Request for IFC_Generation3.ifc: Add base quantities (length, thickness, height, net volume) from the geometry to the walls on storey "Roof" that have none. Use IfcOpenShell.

First a look at what the model holds.

```python
import ifcopenshell
import ifcopenshell.util.element
import ifcopenshell.util.unit

model = ifcopenshell.open("IFC_Generation3.ifc")
print(model.schema)
for unit_type in ("LENGTHUNIT", "AREAUNIT", "VOLUMEUNIT"):
    print(unit_type, ifcopenshell.util.unit.calculate_unit_scale(model, unit_type))
storey = next(s for s in model.by_type("IfcBuildingStorey") if s.Name == "Roof")
walls = [e for e in ifcopenshell.util.element.get_decomposition(storey) if e.is_a("IfcWall")]
for e in sorted(walls, key=lambda e: e.id()):
    print(e.id(), e.is_a(), e.Name, list(ifcopenshell.util.element.get_psets(e, qtos_only=True)), sep=" | ")
```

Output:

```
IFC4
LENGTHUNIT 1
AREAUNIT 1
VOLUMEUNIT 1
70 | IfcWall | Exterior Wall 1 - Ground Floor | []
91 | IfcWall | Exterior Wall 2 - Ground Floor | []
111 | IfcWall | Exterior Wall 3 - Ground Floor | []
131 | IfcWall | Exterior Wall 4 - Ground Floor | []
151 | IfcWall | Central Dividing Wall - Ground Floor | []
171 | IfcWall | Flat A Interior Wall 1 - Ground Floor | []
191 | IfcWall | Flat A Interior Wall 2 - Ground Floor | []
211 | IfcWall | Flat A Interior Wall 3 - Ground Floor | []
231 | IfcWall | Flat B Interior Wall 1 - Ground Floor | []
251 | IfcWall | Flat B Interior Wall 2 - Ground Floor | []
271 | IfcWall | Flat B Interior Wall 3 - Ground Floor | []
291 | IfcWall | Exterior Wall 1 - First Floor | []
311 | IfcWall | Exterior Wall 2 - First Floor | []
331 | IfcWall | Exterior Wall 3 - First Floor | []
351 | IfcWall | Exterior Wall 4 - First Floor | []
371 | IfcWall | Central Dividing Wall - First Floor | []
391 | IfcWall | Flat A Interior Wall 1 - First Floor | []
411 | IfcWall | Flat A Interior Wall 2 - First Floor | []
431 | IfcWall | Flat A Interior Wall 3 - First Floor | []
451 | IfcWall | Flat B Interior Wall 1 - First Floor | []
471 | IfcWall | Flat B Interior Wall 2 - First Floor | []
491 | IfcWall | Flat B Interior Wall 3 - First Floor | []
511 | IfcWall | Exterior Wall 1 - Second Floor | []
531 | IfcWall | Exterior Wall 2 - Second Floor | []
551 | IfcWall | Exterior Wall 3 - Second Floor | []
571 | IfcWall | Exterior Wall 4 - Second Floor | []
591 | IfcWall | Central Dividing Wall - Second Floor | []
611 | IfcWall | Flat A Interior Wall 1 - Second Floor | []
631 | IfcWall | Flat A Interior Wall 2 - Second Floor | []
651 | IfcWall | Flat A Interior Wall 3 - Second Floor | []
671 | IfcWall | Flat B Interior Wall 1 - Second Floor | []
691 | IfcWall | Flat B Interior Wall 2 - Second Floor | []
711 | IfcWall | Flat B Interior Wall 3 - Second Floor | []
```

```python
import ifcopenshell
import ifcopenshell.api.pset
import ifcopenshell.geom
import ifcopenshell.util.element
import ifcopenshell.util.shape
import ifcopenshell.util.unit

model = ifcopenshell.open("IFC_Generation3.ifc")
unit_scale = ifcopenshell.util.unit.calculate_unit_scale(model)
volume_scale = ifcopenshell.util.unit.calculate_unit_scale(model, "VOLUMEUNIT")
settings = ifcopenshell.geom.settings()

storey = next(s for s in model.by_type("IfcBuildingStorey") if s.Name == "Roof")
walls = [e for e in ifcopenshell.util.element.get_decomposition(storey) if e.is_a("IfcWall")]

for e in sorted(walls, key=lambda e: e.id()):
    if ifcopenshell.util.element.get_psets(e, qtos_only=True, should_inherit=False):
        continue
    # Geometry comes back in metres, in the element's own axes.
    shape = ifcopenshell.geom.create_shape(settings, e)
    values = {
        "Length": ifcopenshell.util.shape.get_x(shape.geometry) / unit_scale,
        "Width": ifcopenshell.util.shape.get_y(shape.geometry) / unit_scale,
        "Height": ifcopenshell.util.shape.get_z(shape.geometry) / unit_scale,
        "NetVolume": ifcopenshell.util.shape.get_volume(shape.geometry) / volume_scale,
    }
    qto = ifcopenshell.api.pset.add_qto(model, product=e, name="Qto_WallBaseQuantities")
    ifcopenshell.api.pset.edit_qto(model, qto=qto, properties=values)
    print(e.id(), {k: round(v, 3) for k, v in values.items()})

model.write("IFC_Generation3-out.ifc")
```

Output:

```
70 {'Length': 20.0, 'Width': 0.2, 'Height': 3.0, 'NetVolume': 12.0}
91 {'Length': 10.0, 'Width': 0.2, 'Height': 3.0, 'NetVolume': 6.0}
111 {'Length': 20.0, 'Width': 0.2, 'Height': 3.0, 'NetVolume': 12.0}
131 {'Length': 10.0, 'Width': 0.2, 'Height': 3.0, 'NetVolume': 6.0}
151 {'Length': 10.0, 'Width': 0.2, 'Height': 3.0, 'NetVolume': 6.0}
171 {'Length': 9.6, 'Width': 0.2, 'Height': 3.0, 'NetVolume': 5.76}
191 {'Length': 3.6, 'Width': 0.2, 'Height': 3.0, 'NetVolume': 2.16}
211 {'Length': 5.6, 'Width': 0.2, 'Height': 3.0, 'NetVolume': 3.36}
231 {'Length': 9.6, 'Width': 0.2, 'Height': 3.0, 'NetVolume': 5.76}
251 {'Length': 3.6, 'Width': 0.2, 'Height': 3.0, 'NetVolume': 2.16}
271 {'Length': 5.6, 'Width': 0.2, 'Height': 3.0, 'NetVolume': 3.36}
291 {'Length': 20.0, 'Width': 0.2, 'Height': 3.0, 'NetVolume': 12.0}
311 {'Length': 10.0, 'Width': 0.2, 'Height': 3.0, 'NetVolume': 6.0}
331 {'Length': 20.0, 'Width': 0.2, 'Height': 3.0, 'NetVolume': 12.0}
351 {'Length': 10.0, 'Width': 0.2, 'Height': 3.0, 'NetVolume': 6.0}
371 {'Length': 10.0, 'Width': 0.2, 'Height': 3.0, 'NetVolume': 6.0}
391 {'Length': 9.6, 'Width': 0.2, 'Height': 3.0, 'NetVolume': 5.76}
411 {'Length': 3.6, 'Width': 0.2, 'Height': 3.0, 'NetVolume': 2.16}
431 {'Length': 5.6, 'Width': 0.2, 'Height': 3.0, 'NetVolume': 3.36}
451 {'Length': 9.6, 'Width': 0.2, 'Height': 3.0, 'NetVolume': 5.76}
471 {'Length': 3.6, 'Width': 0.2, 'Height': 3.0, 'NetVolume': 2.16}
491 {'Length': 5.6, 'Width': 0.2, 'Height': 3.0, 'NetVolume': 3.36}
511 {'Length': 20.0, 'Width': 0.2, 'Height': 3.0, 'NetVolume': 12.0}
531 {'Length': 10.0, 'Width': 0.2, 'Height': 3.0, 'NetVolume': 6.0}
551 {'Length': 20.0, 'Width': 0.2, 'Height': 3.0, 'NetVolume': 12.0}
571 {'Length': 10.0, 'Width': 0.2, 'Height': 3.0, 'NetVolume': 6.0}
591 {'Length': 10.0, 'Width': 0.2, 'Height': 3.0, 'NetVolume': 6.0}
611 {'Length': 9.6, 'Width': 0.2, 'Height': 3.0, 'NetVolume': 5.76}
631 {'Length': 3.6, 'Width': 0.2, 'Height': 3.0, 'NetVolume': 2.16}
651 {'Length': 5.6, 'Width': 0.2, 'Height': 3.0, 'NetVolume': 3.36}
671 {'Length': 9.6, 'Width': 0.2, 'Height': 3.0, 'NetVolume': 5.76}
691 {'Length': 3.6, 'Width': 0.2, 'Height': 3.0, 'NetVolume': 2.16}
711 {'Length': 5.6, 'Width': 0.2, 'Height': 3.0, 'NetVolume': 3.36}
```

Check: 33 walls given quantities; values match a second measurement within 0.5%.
